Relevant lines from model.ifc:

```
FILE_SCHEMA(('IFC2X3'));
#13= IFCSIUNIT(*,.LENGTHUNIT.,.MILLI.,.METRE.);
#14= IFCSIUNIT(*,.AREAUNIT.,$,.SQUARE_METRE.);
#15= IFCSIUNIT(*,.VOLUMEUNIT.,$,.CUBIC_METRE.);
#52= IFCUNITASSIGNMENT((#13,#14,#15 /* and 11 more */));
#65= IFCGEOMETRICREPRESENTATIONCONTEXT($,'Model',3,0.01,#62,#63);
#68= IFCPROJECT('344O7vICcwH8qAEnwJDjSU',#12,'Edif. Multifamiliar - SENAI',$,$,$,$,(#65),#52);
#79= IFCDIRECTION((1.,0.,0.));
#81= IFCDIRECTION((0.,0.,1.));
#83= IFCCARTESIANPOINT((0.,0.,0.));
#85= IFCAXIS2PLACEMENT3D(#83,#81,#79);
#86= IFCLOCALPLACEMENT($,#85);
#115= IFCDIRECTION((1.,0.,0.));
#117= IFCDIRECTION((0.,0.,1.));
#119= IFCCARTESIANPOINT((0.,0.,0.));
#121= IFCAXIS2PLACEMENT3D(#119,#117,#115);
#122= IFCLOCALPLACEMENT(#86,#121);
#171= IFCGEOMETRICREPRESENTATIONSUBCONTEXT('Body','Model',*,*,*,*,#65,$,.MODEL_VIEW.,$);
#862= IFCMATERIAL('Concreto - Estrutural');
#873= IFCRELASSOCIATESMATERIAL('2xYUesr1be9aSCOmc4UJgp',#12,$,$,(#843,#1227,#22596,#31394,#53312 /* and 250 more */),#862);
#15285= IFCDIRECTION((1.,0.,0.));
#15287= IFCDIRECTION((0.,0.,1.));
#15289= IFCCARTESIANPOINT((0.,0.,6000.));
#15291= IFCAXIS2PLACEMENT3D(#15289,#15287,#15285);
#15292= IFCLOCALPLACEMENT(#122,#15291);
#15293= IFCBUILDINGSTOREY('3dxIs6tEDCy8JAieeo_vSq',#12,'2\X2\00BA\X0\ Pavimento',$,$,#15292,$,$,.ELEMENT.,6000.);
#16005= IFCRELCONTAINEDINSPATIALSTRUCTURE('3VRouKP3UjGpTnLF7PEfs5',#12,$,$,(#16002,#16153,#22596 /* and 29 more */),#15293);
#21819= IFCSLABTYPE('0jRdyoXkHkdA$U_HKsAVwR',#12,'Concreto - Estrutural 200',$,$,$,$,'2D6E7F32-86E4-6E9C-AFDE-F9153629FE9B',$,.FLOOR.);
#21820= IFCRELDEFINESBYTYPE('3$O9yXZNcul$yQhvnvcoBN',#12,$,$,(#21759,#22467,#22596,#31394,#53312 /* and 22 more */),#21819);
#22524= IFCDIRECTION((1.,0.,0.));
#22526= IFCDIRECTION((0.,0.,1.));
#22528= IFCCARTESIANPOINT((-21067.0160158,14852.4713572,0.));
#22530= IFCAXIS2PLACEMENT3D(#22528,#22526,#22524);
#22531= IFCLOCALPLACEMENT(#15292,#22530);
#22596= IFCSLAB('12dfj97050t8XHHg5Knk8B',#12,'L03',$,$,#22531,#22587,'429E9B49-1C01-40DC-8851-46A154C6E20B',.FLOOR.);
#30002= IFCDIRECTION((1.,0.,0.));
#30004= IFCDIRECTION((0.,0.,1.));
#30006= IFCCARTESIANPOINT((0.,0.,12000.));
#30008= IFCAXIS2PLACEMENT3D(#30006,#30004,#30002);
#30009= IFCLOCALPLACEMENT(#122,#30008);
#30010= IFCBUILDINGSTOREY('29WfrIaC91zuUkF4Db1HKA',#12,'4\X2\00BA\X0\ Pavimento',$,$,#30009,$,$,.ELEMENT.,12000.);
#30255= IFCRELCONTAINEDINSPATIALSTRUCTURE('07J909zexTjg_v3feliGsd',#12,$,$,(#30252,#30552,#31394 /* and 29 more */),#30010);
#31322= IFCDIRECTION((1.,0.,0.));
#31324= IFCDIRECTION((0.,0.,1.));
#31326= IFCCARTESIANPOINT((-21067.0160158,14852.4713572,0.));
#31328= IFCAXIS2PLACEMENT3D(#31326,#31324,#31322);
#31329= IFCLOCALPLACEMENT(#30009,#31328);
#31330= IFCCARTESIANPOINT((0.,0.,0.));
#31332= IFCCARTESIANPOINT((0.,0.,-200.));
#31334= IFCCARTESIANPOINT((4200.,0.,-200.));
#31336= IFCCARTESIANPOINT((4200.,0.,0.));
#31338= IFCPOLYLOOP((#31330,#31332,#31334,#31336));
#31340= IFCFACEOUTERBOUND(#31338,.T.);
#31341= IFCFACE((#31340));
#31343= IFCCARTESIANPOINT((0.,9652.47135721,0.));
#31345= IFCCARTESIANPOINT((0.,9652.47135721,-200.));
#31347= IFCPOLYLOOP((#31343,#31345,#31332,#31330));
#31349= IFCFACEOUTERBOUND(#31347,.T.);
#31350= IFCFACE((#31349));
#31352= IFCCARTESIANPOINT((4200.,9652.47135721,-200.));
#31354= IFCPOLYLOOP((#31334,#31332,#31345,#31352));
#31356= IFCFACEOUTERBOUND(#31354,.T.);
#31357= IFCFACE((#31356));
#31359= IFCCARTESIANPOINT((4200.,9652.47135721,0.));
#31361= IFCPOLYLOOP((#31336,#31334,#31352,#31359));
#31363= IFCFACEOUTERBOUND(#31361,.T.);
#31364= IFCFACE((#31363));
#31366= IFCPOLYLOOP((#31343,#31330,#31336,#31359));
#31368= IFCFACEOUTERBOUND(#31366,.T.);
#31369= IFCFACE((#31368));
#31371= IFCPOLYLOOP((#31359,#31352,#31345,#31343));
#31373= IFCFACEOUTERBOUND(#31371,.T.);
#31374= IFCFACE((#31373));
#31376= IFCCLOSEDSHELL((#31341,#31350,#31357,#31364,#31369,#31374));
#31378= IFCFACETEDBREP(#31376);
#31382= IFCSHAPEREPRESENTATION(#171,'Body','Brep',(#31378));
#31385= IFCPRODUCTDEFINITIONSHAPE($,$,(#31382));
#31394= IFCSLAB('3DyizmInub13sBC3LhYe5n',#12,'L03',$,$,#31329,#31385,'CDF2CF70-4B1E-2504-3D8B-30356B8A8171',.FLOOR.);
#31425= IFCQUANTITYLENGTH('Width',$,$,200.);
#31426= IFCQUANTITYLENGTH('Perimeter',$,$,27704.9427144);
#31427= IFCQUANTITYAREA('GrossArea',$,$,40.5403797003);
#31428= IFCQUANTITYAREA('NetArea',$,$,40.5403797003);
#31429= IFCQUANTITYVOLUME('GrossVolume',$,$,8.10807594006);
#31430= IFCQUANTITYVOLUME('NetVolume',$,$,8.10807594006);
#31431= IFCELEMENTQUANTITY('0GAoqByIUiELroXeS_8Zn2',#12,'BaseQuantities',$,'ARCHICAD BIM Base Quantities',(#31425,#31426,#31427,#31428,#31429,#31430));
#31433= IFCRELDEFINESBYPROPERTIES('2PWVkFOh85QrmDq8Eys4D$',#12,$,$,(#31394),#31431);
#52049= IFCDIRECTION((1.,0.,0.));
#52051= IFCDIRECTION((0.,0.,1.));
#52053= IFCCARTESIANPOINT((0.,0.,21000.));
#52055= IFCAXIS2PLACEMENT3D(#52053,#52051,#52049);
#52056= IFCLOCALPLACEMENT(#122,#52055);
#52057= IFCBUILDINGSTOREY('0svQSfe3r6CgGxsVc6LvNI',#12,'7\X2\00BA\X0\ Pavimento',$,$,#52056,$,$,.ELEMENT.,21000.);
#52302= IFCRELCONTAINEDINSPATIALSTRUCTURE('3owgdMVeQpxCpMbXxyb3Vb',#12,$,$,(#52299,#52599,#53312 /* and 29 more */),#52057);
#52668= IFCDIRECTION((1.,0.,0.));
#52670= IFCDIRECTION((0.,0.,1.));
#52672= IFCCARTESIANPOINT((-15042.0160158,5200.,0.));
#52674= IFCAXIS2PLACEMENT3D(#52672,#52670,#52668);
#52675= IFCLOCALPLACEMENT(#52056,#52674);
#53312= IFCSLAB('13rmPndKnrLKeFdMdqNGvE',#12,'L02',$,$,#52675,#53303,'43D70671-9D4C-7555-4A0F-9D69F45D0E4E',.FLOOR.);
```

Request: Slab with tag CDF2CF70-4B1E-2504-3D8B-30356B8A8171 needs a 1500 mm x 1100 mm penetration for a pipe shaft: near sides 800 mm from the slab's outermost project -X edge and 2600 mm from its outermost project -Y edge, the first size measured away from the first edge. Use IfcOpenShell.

```python
import numpy as np
import ifcopenshell
import ifcopenshell.api.feature
import ifcopenshell.api.geometry
import ifcopenshell.api.pset
import ifcopenshell.api.root
import ifcopenshell.geom
import ifcopenshell.util.element
import ifcopenshell.util.placement
import ifcopenshell.util.representation
import ifcopenshell.util.shape
import ifcopenshell.util.unit

model = ifcopenshell.open("model.ifc")
unit_scale = ifcopenshell.util.unit.calculate_unit_scale(model)
area_scale = ifcopenshell.util.unit.calculate_unit_scale(model, "AREAUNIT")
volume_scale = ifcopenshell.util.unit.calculate_unit_scale(model, "VOLUMEUNIT")
settings = ifcopenshell.geom.settings()


def volume(element):
    """Net volume in cubic metres, openings subtracted."""
    shape = ifcopenshell.geom.create_shape(settings, element)
    return ifcopenshell.util.shape.get_volume(shape.geometry)


slab = model.by_id(31394)
before = volume(slab)

# Extent in the slab's own axes, in metres. The edges named are its -X and -Y sides.
slab_shape = ifcopenshell.geom.create_shape(settings, slab)
vertices = ifcopenshell.util.shape.get_vertices(slab_shape.geometry)
x_min, y_min, bottom = vertices.min(axis=0)
top = vertices[:, 2].max()

opening = ifcopenshell.api.root.create_entity(model, ifc_class="IfcOpeningElement", name="Pipe shaft opening")
context = ifcopenshell.util.representation.get_context(model, "Model", "Body", "MODEL_VIEW")
width, depth = 1.5, 1.1
outline = [(0.0, 0.0), (width, 0.0), (width, depth), (0.0, depth), (0.0, 0.0)]
# Overshoot both faces by 50 mm so the cut is clean.
shape = ifcopenshell.api.geometry.add_slab_representation(
    model, context=context, depth=top - bottom + 0.1, polyline=outline
)
ifcopenshell.api.geometry.assign_representation(model, product=opening, representation=shape)

matrix = ifcopenshell.util.placement.get_local_placement(slab.ObjectPlacement)
matrix[:, 3] = matrix @ np.append(np.array([x_min + 0.8, y_min + 2.6, bottom - 0.05]) / unit_scale, 1.0)
ifcopenshell.api.geometry.edit_object_placement(model, product=opening, matrix=matrix, is_si=False)
ifcopenshell.api.feature.add_feature(model, feature=opening, element=slab)

after = volume(slab)

# Update the slab's stored quantities.
qto = model.by_id(ifcopenshell.util.element.get_pset(slab, "BaseQuantities", should_inherit=False)["id"])
ifcopenshell.api.pset.edit_qto(model, qto=qto, properties={
    "NetArea": after / (top - bottom) / area_scale,
    "NetVolume": after / volume_scale,
})

print(f"slab volume {before:.3f} -> {after:.3f} m3")

model.write("model_rev.ifc")
```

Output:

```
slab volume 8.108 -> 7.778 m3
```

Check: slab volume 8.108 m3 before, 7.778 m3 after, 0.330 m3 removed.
